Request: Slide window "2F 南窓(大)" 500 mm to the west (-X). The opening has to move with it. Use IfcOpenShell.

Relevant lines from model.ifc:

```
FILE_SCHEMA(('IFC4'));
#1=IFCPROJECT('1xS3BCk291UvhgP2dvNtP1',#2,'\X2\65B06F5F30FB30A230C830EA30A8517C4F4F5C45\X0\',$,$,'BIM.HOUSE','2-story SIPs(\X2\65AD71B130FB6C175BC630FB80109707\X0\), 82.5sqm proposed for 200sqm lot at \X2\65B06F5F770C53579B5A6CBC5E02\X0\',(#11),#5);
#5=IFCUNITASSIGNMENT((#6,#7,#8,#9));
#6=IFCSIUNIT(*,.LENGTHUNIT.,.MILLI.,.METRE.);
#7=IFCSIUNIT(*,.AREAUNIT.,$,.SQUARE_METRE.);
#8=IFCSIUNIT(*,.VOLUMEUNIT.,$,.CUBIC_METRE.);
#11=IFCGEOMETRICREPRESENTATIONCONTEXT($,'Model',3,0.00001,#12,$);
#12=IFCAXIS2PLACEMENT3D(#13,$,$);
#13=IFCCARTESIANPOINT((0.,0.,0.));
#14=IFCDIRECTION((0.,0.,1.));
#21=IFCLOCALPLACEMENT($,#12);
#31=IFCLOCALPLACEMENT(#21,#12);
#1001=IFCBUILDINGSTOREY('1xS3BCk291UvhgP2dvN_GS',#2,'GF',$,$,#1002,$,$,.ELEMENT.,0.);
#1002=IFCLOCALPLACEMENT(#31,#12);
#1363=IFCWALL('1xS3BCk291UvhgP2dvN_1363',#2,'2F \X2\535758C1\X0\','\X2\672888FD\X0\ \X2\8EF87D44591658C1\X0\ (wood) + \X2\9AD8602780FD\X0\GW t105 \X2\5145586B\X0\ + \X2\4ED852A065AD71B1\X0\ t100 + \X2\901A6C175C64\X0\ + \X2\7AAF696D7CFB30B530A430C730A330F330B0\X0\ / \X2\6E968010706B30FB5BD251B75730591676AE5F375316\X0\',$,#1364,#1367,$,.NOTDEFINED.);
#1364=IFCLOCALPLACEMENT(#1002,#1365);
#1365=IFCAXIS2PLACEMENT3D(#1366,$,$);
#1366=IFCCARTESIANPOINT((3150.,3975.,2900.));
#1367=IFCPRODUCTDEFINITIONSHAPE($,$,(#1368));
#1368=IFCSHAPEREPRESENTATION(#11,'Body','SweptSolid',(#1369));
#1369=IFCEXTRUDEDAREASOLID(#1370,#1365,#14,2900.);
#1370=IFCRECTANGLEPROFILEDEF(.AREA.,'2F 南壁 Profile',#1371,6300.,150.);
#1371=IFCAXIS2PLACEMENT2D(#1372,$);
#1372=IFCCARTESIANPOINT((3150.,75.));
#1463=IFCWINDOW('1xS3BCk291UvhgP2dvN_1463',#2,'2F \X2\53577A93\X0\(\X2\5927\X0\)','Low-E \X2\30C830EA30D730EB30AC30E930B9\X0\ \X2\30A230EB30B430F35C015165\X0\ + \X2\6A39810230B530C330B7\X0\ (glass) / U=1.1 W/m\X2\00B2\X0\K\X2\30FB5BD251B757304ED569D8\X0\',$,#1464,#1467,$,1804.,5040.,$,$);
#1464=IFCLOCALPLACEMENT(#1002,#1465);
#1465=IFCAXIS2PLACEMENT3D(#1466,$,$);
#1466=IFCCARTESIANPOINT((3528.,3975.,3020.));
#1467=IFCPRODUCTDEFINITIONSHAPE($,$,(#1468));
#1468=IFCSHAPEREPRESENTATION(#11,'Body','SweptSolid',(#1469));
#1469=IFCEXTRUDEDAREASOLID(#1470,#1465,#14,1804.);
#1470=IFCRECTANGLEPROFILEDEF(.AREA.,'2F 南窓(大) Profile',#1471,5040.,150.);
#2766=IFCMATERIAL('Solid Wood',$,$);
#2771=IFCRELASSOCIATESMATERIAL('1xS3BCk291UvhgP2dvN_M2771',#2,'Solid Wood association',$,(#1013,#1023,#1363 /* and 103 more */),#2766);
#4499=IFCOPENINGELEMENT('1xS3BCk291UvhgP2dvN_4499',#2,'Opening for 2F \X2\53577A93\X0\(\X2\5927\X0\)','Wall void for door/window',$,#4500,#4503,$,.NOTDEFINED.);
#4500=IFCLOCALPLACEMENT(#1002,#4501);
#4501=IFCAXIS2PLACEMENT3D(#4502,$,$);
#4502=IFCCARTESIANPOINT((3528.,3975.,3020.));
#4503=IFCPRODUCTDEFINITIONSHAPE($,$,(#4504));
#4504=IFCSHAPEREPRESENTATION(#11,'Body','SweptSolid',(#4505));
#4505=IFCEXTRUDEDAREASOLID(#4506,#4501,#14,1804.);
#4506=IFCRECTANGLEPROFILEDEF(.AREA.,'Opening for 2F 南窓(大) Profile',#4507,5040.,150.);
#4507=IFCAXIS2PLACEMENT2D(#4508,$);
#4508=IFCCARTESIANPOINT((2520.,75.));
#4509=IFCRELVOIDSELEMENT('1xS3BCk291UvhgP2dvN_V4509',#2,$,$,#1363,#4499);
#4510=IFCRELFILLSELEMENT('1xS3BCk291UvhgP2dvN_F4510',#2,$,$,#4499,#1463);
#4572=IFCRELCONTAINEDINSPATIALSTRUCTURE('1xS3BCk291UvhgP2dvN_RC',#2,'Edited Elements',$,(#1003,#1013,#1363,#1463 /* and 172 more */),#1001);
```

```python
import ifcopenshell
import ifcopenshell.api.geometry
import ifcopenshell.util.placement
import ifcopenshell.util.unit

model = ifcopenshell.open("model.ifc")
unit_scale = ifcopenshell.util.unit.calculate_unit_scale(model)

window = model.by_id(1463)
opening = window.FillsVoids[0].RelatingOpeningElement
wall = opening.VoidsElements[0].RelatingBuildingElement

wall_matrix = ifcopenshell.util.placement.get_local_placement(wall.ObjectPlacement)
shift = wall_matrix[:3, 0] * -0.5 / unit_scale
before = ifcopenshell.util.placement.get_local_placement(window.ObjectPlacement)[:3, 3].copy()

# The window is not placed relative to its opening, so move both.
for product in (opening, window):
    matrix = ifcopenshell.util.placement.get_local_placement(product.ObjectPlacement)
    matrix[:3, 3] += shift
    ifcopenshell.api.geometry.edit_object_placement(model, product=product, matrix=matrix, is_si=False)

after = ifcopenshell.util.placement.get_local_placement(window.ObjectPlacement)[:3, 3]
print("window moved by", (after - before).round(3) + 0.0)

model.write("model_edited.ifc")
```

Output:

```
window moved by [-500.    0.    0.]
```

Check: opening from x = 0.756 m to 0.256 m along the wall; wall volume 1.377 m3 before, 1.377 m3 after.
